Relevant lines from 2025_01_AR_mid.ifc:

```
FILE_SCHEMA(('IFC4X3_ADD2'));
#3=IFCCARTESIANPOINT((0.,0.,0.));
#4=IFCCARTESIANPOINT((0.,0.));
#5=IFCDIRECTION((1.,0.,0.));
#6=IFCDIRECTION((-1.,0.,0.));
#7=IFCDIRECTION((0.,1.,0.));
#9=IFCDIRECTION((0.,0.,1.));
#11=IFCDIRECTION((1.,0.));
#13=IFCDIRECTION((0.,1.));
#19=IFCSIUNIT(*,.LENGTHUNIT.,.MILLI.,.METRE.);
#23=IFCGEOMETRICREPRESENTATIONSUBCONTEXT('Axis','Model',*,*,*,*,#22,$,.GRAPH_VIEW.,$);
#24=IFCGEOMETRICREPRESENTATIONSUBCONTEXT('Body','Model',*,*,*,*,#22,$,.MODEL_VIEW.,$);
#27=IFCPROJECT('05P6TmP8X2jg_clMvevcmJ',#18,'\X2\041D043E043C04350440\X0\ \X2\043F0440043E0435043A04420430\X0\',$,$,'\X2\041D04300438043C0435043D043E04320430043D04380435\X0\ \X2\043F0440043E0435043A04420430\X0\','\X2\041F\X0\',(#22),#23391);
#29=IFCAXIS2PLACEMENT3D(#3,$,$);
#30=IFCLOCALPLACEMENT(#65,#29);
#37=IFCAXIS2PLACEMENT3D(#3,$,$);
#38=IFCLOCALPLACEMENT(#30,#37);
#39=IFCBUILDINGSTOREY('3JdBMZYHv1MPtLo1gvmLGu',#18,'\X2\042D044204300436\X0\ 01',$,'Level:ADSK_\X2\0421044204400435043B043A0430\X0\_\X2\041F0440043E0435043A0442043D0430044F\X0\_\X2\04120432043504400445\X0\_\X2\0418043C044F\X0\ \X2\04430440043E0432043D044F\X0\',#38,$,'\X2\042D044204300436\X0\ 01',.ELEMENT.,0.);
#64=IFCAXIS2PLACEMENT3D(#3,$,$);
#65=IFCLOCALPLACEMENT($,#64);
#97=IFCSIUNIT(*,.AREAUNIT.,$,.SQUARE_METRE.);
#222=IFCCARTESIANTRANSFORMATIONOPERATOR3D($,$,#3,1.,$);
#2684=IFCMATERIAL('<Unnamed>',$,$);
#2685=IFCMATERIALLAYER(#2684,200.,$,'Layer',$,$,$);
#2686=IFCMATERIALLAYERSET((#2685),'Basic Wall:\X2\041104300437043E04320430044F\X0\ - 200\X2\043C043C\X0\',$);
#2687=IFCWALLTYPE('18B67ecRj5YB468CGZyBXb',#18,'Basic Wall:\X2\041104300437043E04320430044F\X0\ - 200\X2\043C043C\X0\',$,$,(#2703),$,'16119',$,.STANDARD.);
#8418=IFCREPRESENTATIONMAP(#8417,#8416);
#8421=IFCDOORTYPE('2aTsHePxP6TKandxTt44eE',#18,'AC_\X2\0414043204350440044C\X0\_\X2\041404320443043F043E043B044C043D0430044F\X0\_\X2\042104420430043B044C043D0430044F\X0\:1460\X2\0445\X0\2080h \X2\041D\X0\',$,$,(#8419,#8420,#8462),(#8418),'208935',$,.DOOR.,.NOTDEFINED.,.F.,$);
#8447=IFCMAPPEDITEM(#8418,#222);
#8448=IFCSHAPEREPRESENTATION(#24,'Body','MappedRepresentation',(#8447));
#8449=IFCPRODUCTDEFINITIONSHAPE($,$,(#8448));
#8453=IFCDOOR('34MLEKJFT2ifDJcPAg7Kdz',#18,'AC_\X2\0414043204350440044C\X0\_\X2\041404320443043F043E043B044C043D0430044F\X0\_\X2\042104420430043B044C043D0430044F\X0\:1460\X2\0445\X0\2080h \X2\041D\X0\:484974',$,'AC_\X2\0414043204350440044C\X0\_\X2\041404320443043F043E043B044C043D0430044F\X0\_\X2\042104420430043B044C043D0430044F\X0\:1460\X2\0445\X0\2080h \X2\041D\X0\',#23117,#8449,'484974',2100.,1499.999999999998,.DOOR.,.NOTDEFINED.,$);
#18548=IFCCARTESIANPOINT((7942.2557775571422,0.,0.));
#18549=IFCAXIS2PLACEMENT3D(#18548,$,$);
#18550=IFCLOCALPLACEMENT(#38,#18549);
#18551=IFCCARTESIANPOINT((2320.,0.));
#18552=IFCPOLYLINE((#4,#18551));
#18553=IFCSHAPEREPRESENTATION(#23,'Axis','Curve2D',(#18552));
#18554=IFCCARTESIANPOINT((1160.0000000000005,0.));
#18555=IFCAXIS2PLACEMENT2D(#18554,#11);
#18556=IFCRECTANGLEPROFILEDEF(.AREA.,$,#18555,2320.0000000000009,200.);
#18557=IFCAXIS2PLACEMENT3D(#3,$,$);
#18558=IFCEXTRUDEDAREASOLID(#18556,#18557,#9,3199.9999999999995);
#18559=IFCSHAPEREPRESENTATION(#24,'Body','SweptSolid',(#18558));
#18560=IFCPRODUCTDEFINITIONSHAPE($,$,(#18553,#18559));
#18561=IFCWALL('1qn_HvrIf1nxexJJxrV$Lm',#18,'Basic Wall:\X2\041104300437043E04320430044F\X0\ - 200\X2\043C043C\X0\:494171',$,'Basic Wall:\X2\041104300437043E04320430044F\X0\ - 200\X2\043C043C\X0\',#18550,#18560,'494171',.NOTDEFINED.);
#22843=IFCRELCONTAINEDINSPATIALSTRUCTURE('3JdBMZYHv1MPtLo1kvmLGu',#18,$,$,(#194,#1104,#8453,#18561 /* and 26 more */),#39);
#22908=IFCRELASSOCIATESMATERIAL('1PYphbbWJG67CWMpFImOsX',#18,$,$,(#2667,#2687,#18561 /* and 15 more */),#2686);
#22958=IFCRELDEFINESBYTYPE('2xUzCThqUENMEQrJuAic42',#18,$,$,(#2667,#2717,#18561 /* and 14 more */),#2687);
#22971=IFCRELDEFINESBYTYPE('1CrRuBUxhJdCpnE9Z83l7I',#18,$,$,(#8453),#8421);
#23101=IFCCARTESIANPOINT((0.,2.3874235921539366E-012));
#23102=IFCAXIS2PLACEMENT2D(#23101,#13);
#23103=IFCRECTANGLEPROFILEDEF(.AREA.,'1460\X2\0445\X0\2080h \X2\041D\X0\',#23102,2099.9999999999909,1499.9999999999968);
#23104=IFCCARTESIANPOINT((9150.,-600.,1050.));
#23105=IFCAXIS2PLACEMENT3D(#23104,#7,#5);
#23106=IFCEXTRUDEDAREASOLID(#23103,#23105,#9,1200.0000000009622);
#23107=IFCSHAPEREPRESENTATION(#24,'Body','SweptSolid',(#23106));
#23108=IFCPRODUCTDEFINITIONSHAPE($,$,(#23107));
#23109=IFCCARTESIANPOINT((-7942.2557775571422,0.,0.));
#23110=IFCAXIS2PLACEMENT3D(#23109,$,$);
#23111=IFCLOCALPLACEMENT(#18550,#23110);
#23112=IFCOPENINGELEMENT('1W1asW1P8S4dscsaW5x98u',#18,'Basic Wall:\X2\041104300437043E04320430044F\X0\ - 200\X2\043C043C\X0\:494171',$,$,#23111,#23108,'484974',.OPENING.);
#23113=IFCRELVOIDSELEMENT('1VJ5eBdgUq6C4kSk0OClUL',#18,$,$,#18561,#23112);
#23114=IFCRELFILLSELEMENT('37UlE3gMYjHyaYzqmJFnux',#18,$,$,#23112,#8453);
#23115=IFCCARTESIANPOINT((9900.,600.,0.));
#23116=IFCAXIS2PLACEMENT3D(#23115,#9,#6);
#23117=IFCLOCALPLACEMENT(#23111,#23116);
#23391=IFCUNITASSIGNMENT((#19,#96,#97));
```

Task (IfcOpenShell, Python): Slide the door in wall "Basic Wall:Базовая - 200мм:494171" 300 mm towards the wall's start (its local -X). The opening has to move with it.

```python
import ifcopenshell
import ifcopenshell.api.geometry
import ifcopenshell.util.placement

model = ifcopenshell.open("2025_01_AR_mid.ifc")

door = model.by_guid("34MLEKJFT2ifDJcPAg7Kdz")
opening = door.FillsVoids[0].RelatingOpeningElement
wall = opening.VoidsElements[0].RelatingBuildingElement

wall_matrix = ifcopenshell.util.placement.get_local_placement(wall.ObjectPlacement)
shift = wall_matrix[:3, 0] * -300.0
before = ifcopenshell.util.placement.get_local_placement(door.ObjectPlacement)[:3, 3].copy()

# The door is placed relative to its opening, so it follows when the opening moves.
matrix = ifcopenshell.util.placement.get_local_placement(opening.ObjectPlacement)
matrix[:3, 3] += shift
ifcopenshell.api.geometry.edit_object_placement(
    model, product=opening, matrix=matrix, is_si=False, should_transform_children=True
)

after = ifcopenshell.util.placement.get_local_placement(door.ObjectPlacement)[:3, 3]
print("door moved by", (after - before).round(3) + 0.0)

model.write("2025_01_AR_mid_rev.ifc")
```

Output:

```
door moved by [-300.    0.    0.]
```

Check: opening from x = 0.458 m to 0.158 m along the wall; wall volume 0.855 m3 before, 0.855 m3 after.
